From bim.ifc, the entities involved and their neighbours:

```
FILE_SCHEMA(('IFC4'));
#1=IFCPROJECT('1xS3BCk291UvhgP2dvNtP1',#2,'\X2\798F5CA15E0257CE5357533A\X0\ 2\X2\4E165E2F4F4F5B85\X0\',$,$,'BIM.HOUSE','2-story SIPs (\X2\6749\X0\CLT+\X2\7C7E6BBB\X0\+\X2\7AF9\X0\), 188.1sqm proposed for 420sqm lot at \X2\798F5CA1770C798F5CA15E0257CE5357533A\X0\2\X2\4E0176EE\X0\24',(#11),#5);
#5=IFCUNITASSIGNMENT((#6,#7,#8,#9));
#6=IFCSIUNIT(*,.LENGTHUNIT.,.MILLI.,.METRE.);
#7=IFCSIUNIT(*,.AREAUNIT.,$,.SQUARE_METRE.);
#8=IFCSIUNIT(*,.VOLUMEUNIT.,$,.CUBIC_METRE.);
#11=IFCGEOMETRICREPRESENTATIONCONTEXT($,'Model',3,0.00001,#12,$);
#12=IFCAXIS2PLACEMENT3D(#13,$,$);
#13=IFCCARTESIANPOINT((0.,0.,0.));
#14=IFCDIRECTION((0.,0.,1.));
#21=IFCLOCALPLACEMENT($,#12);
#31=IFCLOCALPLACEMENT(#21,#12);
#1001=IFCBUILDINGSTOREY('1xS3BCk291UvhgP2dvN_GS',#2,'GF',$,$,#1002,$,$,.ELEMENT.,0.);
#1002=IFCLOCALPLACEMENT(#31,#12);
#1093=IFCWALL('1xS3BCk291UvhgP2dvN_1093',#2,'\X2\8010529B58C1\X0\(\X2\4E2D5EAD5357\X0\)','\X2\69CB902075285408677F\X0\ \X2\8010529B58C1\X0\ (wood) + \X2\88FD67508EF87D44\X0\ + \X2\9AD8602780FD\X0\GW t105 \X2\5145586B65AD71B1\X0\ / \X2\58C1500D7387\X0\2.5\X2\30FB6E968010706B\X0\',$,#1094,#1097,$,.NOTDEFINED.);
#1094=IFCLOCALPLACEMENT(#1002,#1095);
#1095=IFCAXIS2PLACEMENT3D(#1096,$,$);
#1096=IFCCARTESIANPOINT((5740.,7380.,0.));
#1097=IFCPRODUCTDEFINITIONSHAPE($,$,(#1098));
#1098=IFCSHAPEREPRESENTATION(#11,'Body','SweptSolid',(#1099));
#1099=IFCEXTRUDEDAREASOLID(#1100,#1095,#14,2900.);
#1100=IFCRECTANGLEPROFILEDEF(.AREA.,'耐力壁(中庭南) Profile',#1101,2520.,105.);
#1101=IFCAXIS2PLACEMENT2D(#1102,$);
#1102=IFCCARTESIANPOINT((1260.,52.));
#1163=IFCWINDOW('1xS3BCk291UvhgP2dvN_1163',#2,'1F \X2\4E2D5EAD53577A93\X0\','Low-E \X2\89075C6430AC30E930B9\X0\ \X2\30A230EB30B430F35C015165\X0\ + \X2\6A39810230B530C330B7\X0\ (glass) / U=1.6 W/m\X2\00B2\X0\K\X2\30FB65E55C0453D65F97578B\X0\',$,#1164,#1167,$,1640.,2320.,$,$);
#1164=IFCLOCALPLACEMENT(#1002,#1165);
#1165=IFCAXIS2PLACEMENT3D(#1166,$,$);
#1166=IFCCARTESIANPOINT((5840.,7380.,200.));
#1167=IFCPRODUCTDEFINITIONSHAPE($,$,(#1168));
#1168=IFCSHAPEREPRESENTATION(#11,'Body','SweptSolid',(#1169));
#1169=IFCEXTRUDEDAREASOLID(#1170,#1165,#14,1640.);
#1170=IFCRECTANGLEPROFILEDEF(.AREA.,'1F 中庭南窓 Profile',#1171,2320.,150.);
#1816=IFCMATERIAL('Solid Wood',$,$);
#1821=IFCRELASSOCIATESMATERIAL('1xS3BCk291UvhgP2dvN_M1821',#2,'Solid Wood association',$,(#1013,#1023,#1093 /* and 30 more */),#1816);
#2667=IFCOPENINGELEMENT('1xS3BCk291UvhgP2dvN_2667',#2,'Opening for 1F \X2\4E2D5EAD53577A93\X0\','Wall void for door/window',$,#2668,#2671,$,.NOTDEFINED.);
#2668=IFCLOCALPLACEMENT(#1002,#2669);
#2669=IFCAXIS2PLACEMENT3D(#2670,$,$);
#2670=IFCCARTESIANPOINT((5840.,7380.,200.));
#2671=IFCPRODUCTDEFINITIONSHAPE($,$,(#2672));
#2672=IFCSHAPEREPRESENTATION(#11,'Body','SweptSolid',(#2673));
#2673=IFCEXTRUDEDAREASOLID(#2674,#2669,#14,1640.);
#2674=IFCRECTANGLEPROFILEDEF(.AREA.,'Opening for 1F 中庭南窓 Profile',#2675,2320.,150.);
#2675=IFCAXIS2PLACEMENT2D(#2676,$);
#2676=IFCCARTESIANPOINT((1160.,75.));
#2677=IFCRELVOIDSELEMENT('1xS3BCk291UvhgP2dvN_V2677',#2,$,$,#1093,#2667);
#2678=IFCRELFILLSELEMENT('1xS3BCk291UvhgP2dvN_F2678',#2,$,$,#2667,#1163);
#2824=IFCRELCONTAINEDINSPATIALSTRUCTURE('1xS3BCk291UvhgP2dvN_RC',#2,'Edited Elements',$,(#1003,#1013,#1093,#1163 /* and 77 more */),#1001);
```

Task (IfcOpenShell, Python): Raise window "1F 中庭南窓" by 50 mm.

```python
import numpy as np
import ifcopenshell
import ifcopenshell.api.geometry
import ifcopenshell.util.placement
import ifcopenshell.util.unit

model = ifcopenshell.open("bim.ifc")
unit_scale = ifcopenshell.util.unit.calculate_unit_scale(model)

window = model.by_guid("1xS3BCk291UvhgP2dvN_1163")
opening = window.FillsVoids[0].RelatingOpeningElement
dz = 0.05 / unit_scale

shift = np.array([0.0, 0.0, dz])
# The window is not placed relative to its opening, so move both.
for product in (opening, window):
    matrix = ifcopenshell.util.placement.get_local_placement(product.ObjectPlacement)
    matrix[:3, 3] += shift
    ifcopenshell.api.geometry.edit_object_placement(model, product=product, matrix=matrix, is_si=False)

print(f"moved by {dz * unit_scale:+.3f} m")

model.write("bim_rev.ifc")
```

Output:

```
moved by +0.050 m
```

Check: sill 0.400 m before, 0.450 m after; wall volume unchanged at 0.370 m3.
